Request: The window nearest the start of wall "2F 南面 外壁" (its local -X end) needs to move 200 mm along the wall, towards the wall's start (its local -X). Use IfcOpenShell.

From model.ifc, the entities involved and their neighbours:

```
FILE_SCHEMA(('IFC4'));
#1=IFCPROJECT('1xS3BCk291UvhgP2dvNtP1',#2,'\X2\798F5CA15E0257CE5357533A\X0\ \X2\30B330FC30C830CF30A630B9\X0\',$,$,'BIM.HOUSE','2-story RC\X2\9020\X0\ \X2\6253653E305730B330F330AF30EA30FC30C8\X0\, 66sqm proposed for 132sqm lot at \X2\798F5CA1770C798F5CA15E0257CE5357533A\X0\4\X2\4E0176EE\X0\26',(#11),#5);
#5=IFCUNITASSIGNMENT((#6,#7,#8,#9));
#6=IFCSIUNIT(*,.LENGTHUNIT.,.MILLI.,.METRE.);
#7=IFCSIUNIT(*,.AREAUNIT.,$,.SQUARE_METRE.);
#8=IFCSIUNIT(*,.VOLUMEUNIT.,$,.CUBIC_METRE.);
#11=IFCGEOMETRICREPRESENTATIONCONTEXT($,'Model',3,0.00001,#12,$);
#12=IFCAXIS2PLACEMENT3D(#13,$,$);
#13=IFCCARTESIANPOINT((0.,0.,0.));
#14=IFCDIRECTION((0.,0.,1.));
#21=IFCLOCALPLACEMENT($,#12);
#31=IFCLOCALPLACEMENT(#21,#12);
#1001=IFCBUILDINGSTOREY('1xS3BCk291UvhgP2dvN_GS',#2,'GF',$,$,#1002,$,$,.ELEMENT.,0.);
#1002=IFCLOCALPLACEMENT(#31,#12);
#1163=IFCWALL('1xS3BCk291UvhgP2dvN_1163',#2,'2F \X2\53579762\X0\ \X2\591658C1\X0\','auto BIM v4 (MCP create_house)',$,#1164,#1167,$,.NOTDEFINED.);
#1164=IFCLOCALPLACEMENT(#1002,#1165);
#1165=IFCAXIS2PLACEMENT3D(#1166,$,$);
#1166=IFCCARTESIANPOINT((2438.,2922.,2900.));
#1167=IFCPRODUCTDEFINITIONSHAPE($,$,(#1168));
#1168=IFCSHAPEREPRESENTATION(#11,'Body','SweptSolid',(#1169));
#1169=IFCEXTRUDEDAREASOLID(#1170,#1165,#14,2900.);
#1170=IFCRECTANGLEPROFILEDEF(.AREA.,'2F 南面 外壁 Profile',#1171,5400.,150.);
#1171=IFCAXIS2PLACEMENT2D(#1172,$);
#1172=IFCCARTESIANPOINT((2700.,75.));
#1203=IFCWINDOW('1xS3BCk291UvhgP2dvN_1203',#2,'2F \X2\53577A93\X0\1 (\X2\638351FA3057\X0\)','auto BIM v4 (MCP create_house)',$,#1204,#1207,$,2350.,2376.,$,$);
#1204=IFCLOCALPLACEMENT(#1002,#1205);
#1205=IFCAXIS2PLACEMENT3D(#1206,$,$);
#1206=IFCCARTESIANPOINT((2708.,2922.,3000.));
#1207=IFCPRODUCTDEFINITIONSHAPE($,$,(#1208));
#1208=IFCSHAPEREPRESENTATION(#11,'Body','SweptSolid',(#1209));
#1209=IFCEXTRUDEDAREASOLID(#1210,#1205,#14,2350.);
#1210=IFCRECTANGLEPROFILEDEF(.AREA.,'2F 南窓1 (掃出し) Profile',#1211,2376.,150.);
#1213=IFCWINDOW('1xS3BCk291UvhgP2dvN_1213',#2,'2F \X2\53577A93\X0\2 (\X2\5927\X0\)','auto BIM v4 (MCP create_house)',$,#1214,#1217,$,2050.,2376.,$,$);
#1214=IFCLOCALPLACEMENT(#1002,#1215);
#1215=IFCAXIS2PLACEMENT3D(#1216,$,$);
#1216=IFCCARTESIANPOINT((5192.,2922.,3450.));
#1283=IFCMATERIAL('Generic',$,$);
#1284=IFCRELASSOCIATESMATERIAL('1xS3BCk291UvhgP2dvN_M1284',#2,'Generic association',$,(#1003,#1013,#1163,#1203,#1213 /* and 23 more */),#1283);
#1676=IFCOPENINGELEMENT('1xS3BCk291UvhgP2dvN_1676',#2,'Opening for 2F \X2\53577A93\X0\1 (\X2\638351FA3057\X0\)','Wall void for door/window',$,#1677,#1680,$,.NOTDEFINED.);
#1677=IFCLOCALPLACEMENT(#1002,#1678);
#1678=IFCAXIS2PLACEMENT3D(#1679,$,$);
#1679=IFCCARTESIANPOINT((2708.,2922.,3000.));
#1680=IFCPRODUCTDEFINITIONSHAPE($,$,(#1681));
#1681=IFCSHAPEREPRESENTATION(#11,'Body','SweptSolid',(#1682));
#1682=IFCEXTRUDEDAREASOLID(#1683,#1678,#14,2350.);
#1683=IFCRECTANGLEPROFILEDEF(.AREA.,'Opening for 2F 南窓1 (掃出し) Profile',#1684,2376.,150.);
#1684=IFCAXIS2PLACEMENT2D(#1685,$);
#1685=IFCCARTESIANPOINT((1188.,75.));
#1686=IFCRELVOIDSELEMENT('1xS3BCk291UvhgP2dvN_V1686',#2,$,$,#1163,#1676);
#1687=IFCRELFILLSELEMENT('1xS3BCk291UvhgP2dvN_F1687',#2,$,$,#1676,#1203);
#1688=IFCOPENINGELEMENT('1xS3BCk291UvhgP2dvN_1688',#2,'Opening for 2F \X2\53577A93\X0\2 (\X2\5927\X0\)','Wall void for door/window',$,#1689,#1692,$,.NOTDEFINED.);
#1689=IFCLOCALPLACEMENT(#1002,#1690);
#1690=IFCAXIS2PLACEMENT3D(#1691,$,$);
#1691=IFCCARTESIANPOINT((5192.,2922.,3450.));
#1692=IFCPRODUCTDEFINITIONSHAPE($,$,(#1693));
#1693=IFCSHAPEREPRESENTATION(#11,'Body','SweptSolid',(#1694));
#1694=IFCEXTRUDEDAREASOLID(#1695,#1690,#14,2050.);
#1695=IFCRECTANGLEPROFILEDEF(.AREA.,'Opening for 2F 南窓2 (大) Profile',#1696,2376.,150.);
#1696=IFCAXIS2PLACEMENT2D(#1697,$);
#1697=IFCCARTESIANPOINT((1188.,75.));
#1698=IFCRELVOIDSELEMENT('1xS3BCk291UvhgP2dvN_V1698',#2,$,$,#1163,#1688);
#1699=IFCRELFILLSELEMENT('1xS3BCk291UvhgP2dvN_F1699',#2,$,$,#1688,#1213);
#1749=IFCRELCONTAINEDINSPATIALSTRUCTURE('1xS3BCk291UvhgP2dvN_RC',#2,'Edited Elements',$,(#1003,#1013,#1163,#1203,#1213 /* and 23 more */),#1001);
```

```python
import ifcopenshell
import ifcopenshell.api.geometry
import ifcopenshell.util.placement
import ifcopenshell.util.unit

model = ifcopenshell.open("model.ifc")
unit_scale = ifcopenshell.util.unit.calculate_unit_scale(model)

window = model.by_guid("1xS3BCk291UvhgP2dvN_1203")
opening = window.FillsVoids[0].RelatingOpeningElement
wall = opening.VoidsElements[0].RelatingBuildingElement

wall_matrix = ifcopenshell.util.placement.get_local_placement(wall.ObjectPlacement)
shift = wall_matrix[:3, 0] * -0.2 / unit_scale
before = ifcopenshell.util.placement.get_local_placement(window.ObjectPlacement)[:3, 3].copy()

# The window is not placed relative to its opening, so move both.
for product in (opening, window):
    matrix = ifcopenshell.util.placement.get_local_placement(product.ObjectPlacement)
    matrix[:3, 3] += shift
    ifcopenshell.api.geometry.edit_object_placement(model, product=product, matrix=matrix, is_si=False)

after = ifcopenshell.util.placement.get_local_placement(window.ObjectPlacement)[:3, 3]
print("window moved by", (after - before).round(3) + 0.0)

model.write("model_v2.ifc")
```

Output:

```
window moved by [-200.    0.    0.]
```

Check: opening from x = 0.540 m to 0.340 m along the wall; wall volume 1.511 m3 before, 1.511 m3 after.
